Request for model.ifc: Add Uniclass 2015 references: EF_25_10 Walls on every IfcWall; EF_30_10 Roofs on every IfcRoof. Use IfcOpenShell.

First a look at what the model holds.

```python
import ifcopenshell

model = ifcopenshell.open("model.ifc")
print(model.schema)
print("classifications:", [c.Name for c in model.by_type("IfcClassification")])
for ifc_class in ("IfcDoor", "IfcRoof", "IfcStair", "IfcWall", "IfcWindow"):
    print(ifc_class, len(model.by_type(ifc_class)))
```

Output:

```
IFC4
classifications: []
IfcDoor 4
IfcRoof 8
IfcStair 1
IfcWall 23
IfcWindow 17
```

```python
import ifcopenshell
import ifcopenshell.api.classification

model = ifcopenshell.open("model.ifc")

system = ifcopenshell.api.classification.add_classification(model, classification="Uniclass 2015")

codes = {
    "IfcWall": ("EF_25_10", "Walls"),
    "IfcRoof": ("EF_30_10", "Roofs"),
}
for ifc_class, (code, name) in codes.items():
    products = model.by_type(ifc_class)
    ifcopenshell.api.classification.add_reference(
        model, products=products, classification=system, identification=code, name=name
    )
    print(code, len(products))

model.write("model_rev.ifc")
```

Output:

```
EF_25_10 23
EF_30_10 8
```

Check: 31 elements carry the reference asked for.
